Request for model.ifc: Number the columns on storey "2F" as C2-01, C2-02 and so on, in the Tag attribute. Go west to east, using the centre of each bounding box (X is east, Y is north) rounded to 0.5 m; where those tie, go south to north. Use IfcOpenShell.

First a look at what the model holds.

```python
import ifcopenshell
import ifcopenshell.util.element
import ifcopenshell.util.placement

model = ifcopenshell.open("model.ifc")
print(model.schema)
storey = next(s for s in model.by_type("IfcBuildingStorey") if s.Name == "2F")
columns = [e for e in ifcopenshell.util.element.get_decomposition(storey) if e.is_a("IfcColumn")]
for e in sorted(columns, key=lambda e: e.id()):
    origin = ifcopenshell.util.placement.get_local_placement(e.ObjectPlacement)[:3, 3]
    print(e.id(), e.Tag, e.Name, origin.round(2) + 0.0, sep=" | ")
```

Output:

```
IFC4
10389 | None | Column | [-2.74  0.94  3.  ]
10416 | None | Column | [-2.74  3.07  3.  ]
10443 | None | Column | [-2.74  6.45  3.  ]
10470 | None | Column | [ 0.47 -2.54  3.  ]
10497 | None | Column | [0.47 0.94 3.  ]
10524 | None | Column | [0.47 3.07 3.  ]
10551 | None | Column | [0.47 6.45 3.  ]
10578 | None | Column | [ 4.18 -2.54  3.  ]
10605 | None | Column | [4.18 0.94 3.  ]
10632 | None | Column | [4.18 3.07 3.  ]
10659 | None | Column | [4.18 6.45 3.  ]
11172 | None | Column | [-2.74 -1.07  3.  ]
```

```python
import ifcopenshell
import ifcopenshell.geom
import ifcopenshell.util.element
import ifcopenshell.util.shape

model = ifcopenshell.open("model.ifc")
settings = ifcopenshell.geom.settings()
settings.set("use-world-coords", True)


def centre(element):
    shape = ifcopenshell.geom.create_shape(settings, element)
    return ifcopenshell.util.shape.get_bbox_centroid(shape.geometry)


storey = next(s for s in model.by_type("IfcBuildingStorey") if s.Name == "2F")
columns = [e for e in ifcopenshell.util.element.get_decomposition(storey) if e.is_a("IfcColumn")]

# Insertion points can sit at a corner or the storey origin, so sort by the geometry (in metres).
centres = {e: centre(e) for e in columns}
columns.sort(key=lambda e: (round(centres[e][0] / 0.5), centres[e][1]))

for i, e in enumerate(columns, start=1):
    number = f"C2-{i:02d}"
    e.Tag = number
    print(e.id(), number)

model.write("model-out.ifc")
```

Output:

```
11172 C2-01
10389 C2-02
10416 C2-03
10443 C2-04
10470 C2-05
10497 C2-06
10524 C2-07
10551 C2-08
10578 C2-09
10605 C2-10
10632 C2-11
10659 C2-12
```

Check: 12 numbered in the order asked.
